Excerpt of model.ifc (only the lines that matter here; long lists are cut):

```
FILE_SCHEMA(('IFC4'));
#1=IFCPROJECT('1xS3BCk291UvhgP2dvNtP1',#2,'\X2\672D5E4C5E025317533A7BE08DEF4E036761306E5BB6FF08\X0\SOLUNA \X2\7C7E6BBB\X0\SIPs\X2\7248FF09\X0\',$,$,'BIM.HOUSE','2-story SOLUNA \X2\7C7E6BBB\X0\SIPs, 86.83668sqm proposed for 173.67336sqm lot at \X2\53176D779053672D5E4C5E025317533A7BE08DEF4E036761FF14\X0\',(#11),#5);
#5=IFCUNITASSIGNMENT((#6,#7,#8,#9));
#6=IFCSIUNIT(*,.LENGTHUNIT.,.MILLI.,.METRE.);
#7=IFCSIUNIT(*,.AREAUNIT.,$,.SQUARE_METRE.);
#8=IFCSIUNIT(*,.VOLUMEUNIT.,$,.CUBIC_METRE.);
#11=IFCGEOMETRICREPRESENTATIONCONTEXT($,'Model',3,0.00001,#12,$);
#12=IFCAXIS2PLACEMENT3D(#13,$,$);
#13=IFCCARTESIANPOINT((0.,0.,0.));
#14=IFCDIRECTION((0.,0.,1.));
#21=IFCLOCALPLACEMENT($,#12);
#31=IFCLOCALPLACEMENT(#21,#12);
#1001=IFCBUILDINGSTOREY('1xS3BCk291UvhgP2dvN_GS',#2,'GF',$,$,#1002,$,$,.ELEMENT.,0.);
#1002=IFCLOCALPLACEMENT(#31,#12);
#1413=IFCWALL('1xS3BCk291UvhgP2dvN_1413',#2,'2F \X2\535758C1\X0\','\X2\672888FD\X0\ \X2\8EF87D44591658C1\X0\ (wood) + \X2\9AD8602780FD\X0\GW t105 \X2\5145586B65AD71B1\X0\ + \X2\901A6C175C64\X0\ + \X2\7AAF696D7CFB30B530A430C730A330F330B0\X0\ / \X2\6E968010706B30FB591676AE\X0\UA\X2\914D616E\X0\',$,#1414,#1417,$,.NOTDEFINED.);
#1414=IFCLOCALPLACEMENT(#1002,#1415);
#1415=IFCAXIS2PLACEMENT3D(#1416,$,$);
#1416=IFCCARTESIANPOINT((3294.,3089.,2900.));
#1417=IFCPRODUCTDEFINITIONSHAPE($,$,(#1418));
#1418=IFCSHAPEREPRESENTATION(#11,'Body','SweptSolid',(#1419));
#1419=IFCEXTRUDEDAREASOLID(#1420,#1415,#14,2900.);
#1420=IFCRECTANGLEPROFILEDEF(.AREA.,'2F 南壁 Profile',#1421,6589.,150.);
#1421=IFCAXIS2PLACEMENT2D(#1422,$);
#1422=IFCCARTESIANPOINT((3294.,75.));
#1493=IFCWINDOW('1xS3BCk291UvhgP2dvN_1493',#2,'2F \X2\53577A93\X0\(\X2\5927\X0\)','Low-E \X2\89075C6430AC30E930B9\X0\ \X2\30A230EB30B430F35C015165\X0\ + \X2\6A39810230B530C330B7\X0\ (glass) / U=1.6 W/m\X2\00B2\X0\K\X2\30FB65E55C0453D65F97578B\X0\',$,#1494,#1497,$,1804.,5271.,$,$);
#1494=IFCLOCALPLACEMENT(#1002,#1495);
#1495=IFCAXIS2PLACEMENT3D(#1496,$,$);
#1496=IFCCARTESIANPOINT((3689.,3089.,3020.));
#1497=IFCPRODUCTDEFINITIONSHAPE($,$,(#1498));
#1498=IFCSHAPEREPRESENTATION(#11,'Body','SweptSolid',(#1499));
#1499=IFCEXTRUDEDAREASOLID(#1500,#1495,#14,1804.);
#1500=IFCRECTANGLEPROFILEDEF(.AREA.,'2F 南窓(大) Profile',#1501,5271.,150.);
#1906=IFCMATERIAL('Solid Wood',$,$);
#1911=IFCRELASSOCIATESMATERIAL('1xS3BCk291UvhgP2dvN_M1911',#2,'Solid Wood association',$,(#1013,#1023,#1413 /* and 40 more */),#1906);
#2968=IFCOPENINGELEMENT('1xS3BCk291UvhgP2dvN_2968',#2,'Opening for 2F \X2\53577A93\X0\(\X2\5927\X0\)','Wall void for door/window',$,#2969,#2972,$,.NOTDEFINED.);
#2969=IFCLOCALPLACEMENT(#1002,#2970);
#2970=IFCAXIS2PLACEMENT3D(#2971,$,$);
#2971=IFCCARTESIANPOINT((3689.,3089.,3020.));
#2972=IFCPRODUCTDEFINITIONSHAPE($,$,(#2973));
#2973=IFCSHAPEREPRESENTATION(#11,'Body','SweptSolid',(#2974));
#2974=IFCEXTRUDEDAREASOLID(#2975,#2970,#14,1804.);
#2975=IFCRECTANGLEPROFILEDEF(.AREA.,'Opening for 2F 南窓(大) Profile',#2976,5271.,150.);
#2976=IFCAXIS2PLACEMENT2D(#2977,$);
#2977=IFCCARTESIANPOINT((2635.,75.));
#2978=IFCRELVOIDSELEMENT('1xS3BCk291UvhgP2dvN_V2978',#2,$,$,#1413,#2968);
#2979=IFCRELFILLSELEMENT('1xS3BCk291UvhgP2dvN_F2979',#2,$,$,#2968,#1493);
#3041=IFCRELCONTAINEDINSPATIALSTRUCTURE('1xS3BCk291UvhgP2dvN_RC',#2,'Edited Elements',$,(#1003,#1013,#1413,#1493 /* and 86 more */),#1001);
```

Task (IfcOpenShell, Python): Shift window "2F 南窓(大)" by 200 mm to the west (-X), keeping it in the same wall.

```python
import ifcopenshell
import ifcopenshell.api.geometry
import ifcopenshell.util.placement
import ifcopenshell.util.unit

model = ifcopenshell.open("model.ifc")
unit_scale = ifcopenshell.util.unit.calculate_unit_scale(model)

window = model.by_guid("1xS3BCk291UvhgP2dvN_1493")
opening = window.FillsVoids[0].RelatingOpeningElement
wall = opening.VoidsElements[0].RelatingBuildingElement

wall_matrix = ifcopenshell.util.placement.get_local_placement(wall.ObjectPlacement)
shift = wall_matrix[:3, 0] * -0.2 / unit_scale
before = ifcopenshell.util.placement.get_local_placement(window.ObjectPlacement)[:3, 3].copy()

# The window is not placed relative to its opening, so move both.
for product in (opening, window):
    matrix = ifcopenshell.util.placement.get_local_placement(product.ObjectPlacement)
    matrix[:3, 3] += shift
    ifcopenshell.api.geometry.edit_object_placement(model, product=product, matrix=matrix, is_si=False)

after = ifcopenshell.util.placement.get_local_placement(window.ObjectPlacement)[:3, 3]
print("window moved by", (after - before).round(3) + 0.0)

model.write("model_rev.ifc")
```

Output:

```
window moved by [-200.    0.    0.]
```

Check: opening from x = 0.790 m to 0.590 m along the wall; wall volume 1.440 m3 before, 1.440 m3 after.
